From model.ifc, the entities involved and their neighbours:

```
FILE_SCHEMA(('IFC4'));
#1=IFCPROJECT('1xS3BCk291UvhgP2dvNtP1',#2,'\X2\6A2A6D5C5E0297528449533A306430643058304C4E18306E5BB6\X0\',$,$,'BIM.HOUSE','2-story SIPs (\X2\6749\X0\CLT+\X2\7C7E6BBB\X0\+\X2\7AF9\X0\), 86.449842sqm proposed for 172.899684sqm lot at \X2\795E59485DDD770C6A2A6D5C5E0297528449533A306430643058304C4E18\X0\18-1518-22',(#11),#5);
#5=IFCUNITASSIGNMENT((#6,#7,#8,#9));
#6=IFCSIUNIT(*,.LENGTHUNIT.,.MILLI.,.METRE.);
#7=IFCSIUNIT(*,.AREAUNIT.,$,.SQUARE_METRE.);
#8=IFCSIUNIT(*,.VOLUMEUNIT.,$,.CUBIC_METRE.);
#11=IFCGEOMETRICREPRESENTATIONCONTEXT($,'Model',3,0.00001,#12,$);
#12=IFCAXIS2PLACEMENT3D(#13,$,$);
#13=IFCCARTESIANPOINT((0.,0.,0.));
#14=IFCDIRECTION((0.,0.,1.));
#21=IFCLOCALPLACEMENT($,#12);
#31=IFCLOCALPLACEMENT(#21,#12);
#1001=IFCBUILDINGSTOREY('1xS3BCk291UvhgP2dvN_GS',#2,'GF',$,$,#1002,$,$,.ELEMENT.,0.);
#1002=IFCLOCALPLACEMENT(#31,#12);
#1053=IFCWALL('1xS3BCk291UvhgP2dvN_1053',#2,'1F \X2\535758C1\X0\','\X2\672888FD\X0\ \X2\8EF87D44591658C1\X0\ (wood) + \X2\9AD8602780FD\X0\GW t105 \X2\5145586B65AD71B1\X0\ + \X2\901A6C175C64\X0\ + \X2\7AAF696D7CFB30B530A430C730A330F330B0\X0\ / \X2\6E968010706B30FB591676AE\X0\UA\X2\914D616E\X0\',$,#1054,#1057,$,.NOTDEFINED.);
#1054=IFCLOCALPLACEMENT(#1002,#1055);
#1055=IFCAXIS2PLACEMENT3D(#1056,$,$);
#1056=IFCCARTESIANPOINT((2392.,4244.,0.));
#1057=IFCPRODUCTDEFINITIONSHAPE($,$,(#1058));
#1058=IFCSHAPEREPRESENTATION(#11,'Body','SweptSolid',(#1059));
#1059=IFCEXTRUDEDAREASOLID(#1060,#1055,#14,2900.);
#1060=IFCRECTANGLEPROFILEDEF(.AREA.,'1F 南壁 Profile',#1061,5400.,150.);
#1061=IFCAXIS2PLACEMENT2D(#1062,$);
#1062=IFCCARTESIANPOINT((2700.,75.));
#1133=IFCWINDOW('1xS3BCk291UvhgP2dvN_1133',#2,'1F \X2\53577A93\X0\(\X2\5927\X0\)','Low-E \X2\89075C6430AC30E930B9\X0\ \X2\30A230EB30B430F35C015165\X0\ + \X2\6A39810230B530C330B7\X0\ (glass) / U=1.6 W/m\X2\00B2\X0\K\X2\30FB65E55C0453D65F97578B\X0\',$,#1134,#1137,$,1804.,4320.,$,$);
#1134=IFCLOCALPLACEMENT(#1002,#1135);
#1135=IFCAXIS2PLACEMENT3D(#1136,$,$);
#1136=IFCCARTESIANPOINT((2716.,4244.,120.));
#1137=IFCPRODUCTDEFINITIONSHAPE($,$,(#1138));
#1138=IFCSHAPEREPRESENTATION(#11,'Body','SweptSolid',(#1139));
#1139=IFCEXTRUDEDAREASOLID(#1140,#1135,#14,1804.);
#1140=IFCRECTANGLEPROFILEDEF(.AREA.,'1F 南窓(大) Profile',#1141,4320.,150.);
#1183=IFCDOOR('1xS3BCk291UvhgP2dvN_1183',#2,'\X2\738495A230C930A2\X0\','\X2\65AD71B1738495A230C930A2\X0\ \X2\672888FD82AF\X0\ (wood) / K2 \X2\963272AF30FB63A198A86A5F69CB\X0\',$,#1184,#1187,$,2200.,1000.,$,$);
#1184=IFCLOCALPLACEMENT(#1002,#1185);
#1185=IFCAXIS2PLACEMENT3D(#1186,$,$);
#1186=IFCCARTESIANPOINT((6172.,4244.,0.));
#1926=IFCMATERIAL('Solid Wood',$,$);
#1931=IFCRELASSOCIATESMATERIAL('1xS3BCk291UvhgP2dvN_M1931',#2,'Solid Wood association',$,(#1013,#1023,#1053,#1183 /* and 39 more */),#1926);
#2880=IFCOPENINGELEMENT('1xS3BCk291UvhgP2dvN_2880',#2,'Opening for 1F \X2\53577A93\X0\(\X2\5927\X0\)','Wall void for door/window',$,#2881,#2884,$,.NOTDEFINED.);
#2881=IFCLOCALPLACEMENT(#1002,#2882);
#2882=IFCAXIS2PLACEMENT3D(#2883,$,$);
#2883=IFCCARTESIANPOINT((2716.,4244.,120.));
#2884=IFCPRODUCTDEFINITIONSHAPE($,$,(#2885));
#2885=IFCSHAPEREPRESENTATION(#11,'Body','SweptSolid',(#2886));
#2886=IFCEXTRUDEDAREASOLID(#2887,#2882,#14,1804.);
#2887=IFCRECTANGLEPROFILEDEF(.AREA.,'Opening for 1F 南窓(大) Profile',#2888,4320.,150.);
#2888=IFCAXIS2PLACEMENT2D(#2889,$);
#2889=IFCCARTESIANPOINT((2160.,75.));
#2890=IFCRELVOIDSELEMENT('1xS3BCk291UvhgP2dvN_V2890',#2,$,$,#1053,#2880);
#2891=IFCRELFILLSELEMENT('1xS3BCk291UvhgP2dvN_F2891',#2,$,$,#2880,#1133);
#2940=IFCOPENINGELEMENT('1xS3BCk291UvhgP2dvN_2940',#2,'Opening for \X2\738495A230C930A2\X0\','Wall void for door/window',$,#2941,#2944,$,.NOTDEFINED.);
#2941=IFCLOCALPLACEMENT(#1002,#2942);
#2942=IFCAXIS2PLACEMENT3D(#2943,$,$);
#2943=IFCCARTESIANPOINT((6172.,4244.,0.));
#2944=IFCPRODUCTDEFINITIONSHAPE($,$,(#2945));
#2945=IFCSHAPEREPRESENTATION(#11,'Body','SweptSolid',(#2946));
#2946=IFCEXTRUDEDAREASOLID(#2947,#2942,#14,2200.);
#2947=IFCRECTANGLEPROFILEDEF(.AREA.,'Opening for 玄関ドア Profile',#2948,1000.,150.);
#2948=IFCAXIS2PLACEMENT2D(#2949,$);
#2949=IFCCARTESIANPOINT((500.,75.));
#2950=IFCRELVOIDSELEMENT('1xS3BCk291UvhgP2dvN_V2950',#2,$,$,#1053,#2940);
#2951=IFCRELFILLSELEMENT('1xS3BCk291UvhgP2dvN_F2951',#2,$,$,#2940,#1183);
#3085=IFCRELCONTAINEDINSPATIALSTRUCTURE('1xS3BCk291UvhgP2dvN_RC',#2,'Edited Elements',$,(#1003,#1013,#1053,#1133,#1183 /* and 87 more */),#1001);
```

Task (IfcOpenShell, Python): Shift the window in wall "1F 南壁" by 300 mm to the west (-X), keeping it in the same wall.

```python
import ifcopenshell
import ifcopenshell.api.geometry
import ifcopenshell.util.placement
import ifcopenshell.util.unit

model = ifcopenshell.open("model.ifc")
unit_scale = ifcopenshell.util.unit.calculate_unit_scale(model)

window = model.by_id(1133)
opening = window.FillsVoids[0].RelatingOpeningElement
wall = opening.VoidsElements[0].RelatingBuildingElement

wall_matrix = ifcopenshell.util.placement.get_local_placement(wall.ObjectPlacement)
shift = wall_matrix[:3, 0] * -0.3 / unit_scale
before = ifcopenshell.util.placement.get_local_placement(window.ObjectPlacement)[:3, 3].copy()

# The window is not placed relative to its opening, so move both.
for product in (opening, window):
    matrix = ifcopenshell.util.placement.get_local_placement(product.ObjectPlacement)
    matrix[:3, 3] += shift
    ifcopenshell.api.geometry.edit_object_placement(model, product=product, matrix=matrix, is_si=False)

after = ifcopenshell.util.placement.get_local_placement(window.ObjectPlacement)[:3, 3]
print("window moved by", (after - before).round(3) + 0.0)

model.write("model_rev.ifc")
```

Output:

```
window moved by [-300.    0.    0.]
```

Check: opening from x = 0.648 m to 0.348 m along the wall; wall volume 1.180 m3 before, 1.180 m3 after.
